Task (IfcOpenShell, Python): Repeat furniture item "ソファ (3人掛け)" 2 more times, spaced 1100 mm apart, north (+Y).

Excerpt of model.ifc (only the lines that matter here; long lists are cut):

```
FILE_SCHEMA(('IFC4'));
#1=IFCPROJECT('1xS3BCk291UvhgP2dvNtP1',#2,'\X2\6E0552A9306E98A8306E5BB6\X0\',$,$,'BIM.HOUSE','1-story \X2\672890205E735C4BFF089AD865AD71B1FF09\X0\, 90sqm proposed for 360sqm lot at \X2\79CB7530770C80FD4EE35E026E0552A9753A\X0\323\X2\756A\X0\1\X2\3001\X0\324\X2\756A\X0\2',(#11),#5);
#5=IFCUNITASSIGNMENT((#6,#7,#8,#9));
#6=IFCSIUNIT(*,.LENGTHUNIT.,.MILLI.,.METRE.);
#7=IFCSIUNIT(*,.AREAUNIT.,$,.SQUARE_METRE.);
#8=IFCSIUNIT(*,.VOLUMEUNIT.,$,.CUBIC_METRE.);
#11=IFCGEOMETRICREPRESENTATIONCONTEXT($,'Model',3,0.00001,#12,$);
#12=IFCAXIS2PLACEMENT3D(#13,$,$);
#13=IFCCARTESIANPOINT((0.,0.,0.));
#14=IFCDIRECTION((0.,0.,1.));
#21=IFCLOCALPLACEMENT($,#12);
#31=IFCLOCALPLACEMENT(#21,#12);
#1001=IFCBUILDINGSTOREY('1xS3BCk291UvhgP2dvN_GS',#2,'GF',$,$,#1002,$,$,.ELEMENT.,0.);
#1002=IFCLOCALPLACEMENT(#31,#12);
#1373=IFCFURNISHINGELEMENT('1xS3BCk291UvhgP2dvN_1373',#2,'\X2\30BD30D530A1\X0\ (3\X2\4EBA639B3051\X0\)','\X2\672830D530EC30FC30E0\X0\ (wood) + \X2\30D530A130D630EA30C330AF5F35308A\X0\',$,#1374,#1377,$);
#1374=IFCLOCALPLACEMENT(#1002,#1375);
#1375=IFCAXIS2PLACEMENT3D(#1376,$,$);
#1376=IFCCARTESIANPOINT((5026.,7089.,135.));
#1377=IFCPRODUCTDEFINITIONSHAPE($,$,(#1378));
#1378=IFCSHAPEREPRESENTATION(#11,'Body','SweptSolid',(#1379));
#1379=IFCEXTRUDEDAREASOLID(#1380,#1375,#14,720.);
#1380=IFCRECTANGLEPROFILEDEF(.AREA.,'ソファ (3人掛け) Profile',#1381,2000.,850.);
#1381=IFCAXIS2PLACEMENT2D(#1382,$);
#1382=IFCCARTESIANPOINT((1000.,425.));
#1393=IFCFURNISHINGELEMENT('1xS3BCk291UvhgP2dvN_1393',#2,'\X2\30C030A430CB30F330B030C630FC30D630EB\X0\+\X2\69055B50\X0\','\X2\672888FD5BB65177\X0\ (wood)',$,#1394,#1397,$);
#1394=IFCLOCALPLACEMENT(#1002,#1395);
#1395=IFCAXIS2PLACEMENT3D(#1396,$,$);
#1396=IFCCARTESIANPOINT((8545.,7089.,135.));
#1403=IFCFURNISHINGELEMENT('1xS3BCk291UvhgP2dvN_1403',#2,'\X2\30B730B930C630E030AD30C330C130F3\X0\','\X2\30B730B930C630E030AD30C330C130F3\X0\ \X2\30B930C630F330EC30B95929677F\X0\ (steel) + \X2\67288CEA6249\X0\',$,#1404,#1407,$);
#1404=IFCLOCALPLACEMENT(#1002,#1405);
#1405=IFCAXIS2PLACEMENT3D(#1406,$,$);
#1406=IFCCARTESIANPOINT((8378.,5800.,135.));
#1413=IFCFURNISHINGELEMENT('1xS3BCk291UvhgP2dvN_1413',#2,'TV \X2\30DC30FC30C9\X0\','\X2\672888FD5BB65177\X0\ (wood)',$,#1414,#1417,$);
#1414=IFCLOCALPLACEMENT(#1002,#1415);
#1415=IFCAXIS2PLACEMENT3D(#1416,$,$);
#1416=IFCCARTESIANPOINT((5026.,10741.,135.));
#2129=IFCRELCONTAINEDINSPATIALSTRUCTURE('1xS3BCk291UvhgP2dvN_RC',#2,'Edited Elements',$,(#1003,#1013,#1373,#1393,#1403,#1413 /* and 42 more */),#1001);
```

```python
import numpy as np
import ifcopenshell
import ifcopenshell.api.geometry
import ifcopenshell.api.root
import ifcopenshell.util.element
import ifcopenshell.util.placement
import ifcopenshell.util.unit

model = ifcopenshell.open("model.ifc")
unit_scale = ifcopenshell.util.unit.calculate_unit_scale(model)


def reuse_history(source, copy):
    """copy_class also copies each property set's owner history, people and application; keep the originals."""
    for rel in copy.IsDefinedBy:
        if rel.is_a("IfcRelDefinesByProperties") and (history := rel.RelatingPropertyDefinition.OwnerHistory):
            rel.RelatingPropertyDefinition.OwnerHistory = source.OwnerHistory
            ifcopenshell.util.element.remove_deep2(model, history)


source = model.by_guid("1xS3BCk291UvhgP2dvN_1373")
base = ifcopenshell.util.placement.get_local_placement(source.ObjectPlacement)
step = np.array([0.0, 1.0, 0.0]) * 1.1 / unit_scale

for i in range(1, 3):
    copy = ifcopenshell.api.root.copy_class(model, product=source)
    copy.Representation = ifcopenshell.util.element.copy_deep(
        model, source.Representation, exclude=["IfcGeometricRepresentationContext", "IfcRepresentationMap"]
    )
    reuse_history(source, copy)
    matrix = base.copy()
    matrix[:3, 3] += i * step
    print("added at", matrix[:3, 3].round(3) + 0.0)
    ifcopenshell.api.geometry.edit_object_placement(model, product=copy, matrix=matrix, is_si=False)

model.write("model_v2.ifc")
```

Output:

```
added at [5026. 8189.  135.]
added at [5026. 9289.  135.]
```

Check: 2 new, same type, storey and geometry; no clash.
